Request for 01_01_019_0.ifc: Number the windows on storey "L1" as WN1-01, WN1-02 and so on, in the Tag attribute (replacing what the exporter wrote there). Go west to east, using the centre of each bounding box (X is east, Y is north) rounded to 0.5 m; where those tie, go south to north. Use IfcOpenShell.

First a look at what the model holds.

```python
import ifcopenshell
import ifcopenshell.util.element
import ifcopenshell.util.placement

model = ifcopenshell.open("01_01_019_0.ifc")
print(model.schema)
storey = next(s for s in model.by_type("IfcBuildingStorey") if s.Name == "L1")
windows = [e for e in ifcopenshell.util.element.get_decomposition(storey) if e.is_a("IfcWindow")]
for e in sorted(windows, key=lambda e: e.id()):
    origin = ifcopenshell.util.placement.get_local_placement(e.ObjectPlacement)[:3, 3]
    print(e.id(), e.Tag, e.Name, origin.round(2) + 0.0, sep=" | ")
```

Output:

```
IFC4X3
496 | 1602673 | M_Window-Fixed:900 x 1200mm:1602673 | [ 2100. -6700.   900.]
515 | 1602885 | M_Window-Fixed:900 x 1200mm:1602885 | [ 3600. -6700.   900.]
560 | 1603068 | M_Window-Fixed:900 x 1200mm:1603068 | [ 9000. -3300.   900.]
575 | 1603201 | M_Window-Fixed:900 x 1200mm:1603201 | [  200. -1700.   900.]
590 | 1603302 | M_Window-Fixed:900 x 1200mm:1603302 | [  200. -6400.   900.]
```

```python
import ifcopenshell
import ifcopenshell.geom
import ifcopenshell.util.element
import ifcopenshell.util.shape

model = ifcopenshell.open("01_01_019_0.ifc")
settings = ifcopenshell.geom.settings()
settings.set("use-world-coords", True)


def centre(element):
    shape = ifcopenshell.geom.create_shape(settings, element)
    return ifcopenshell.util.shape.get_bbox_centroid(shape.geometry)


storey = next(s for s in model.by_type("IfcBuildingStorey") if s.Name == "L1")
windows = [e for e in ifcopenshell.util.element.get_decomposition(storey) if e.is_a("IfcWindow")]

# Insertion points can sit at a corner or the storey origin, so sort by the geometry (in metres).
centres = {e: centre(e) for e in windows}
windows.sort(key=lambda e: (round(centres[e][0] / 0.5), centres[e][1]))

for i, e in enumerate(windows, start=1):
    number = f"WN1-{i:02d}"
    e.Tag = number
    print(e.id(), number)

model.write("01_01_019_0_v2.ifc")
```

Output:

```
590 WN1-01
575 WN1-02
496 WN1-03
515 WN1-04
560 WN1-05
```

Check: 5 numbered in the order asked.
